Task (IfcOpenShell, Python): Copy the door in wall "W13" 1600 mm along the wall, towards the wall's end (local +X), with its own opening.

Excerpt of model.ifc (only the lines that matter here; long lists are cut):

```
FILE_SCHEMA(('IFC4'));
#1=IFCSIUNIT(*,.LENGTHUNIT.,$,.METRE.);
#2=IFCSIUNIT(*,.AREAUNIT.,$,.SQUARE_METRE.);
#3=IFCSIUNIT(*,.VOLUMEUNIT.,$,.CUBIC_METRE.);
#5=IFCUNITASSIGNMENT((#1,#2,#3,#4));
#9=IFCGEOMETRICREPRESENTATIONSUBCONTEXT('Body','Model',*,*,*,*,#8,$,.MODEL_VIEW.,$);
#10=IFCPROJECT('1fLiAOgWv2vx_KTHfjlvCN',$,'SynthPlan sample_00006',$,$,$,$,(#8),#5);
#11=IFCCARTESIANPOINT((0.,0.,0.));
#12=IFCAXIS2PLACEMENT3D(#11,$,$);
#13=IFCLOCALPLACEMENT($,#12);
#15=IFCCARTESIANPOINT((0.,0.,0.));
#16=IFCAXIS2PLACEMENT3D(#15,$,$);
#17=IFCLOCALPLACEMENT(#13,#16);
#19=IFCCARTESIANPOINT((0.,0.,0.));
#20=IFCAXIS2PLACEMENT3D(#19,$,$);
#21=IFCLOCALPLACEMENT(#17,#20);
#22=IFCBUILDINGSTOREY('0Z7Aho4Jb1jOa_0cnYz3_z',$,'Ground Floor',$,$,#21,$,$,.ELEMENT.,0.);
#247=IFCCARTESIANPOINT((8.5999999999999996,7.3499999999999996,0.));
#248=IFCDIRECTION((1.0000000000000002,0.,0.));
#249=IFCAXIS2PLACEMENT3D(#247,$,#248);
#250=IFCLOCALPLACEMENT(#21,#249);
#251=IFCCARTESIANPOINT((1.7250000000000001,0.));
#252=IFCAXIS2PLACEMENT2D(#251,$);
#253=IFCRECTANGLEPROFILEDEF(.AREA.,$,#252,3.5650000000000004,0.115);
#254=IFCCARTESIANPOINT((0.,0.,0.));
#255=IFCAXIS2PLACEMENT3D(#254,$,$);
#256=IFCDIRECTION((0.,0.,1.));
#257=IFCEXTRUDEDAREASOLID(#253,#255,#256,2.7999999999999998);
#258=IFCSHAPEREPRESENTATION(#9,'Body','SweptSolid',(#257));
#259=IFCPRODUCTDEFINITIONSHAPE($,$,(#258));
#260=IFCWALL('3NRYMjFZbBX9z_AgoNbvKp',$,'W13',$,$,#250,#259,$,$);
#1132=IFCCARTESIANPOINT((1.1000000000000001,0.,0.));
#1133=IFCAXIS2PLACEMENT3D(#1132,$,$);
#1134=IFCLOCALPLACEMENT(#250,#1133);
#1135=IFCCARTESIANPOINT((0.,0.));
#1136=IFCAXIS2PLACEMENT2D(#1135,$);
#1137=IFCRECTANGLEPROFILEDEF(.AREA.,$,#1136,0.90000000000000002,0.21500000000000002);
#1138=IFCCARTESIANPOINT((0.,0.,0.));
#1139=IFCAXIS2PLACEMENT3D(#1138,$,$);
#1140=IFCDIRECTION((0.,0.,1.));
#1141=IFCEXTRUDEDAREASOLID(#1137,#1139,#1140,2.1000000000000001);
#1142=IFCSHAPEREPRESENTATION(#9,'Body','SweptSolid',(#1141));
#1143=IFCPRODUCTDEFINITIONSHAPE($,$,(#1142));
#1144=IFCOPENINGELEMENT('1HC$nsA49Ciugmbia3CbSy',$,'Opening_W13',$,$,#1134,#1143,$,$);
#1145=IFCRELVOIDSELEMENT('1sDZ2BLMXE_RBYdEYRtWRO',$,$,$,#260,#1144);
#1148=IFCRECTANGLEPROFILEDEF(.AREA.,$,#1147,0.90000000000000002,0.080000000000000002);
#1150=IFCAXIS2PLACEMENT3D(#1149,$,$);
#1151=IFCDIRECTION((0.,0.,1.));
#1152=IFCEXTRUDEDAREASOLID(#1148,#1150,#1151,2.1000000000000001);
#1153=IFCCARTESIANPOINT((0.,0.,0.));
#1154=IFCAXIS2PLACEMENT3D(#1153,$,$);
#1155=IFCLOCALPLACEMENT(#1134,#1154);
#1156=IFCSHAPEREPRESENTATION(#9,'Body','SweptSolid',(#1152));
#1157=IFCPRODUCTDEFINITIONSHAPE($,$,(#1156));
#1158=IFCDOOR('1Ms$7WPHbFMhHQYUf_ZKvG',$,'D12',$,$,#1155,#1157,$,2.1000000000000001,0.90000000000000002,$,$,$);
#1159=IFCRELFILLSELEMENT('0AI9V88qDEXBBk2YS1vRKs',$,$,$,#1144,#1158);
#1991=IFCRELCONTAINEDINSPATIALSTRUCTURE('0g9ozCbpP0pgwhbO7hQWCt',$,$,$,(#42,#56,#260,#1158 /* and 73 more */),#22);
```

```python
import ifcopenshell
import ifcopenshell.api.feature
import ifcopenshell.api.geometry
import ifcopenshell.api.root
import ifcopenshell.geom
import ifcopenshell.util.element
import ifcopenshell.util.placement
import ifcopenshell.util.shape
import ifcopenshell.util.unit

model = ifcopenshell.open("model.ifc")
unit_scale = ifcopenshell.util.unit.calculate_unit_scale(model)
settings = ifcopenshell.geom.settings()


def volume(element):
    """Net volume in cubic metres, openings subtracted."""
    shape = ifcopenshell.geom.create_shape(settings, element)
    return ifcopenshell.util.shape.get_volume(shape.geometry)


door = model.by_guid("1Ms$7WPHbFMhHQYUf_ZKvG")
opening = door.FillsVoids[0].RelatingOpeningElement
wall = opening.VoidsElements[0].RelatingBuildingElement
before = volume(wall)
shift = ifcopenshell.util.placement.get_local_placement(wall.ObjectPlacement)[:3, 0] * 1.6 / unit_scale

# copy_class copies the void relationship, type, container and properties, but no geometry.
new_opening = ifcopenshell.api.root.copy_class(model, product=opening)
new_opening.Representation = ifcopenshell.util.element.copy_deep(
    model, opening.Representation, exclude=["IfcGeometricRepresentationContext", "IfcRepresentationMap"]
)
new_door = ifcopenshell.api.root.copy_class(model, product=door)
new_door.Representation = ifcopenshell.util.element.copy_deep(
    model, door.Representation, exclude=["IfcGeometricRepresentationContext", "IfcRepresentationMap"]
)
ifcopenshell.api.feature.add_filling(model, opening=new_opening, element=new_door)

for old, new in ((opening, new_opening), (door, new_door)):
    matrix = ifcopenshell.util.placement.get_local_placement(old.ObjectPlacement)
    matrix[:3, 3] += shift
    ifcopenshell.api.geometry.edit_object_placement(model, product=new, matrix=matrix, is_si=False)

after = volume(wall)

print(f"wall volume {before:.3f} -> {after:.3f} m3")

model.write("model_v2.ifc")
```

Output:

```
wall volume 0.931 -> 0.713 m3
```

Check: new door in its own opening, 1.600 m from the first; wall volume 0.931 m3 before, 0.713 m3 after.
